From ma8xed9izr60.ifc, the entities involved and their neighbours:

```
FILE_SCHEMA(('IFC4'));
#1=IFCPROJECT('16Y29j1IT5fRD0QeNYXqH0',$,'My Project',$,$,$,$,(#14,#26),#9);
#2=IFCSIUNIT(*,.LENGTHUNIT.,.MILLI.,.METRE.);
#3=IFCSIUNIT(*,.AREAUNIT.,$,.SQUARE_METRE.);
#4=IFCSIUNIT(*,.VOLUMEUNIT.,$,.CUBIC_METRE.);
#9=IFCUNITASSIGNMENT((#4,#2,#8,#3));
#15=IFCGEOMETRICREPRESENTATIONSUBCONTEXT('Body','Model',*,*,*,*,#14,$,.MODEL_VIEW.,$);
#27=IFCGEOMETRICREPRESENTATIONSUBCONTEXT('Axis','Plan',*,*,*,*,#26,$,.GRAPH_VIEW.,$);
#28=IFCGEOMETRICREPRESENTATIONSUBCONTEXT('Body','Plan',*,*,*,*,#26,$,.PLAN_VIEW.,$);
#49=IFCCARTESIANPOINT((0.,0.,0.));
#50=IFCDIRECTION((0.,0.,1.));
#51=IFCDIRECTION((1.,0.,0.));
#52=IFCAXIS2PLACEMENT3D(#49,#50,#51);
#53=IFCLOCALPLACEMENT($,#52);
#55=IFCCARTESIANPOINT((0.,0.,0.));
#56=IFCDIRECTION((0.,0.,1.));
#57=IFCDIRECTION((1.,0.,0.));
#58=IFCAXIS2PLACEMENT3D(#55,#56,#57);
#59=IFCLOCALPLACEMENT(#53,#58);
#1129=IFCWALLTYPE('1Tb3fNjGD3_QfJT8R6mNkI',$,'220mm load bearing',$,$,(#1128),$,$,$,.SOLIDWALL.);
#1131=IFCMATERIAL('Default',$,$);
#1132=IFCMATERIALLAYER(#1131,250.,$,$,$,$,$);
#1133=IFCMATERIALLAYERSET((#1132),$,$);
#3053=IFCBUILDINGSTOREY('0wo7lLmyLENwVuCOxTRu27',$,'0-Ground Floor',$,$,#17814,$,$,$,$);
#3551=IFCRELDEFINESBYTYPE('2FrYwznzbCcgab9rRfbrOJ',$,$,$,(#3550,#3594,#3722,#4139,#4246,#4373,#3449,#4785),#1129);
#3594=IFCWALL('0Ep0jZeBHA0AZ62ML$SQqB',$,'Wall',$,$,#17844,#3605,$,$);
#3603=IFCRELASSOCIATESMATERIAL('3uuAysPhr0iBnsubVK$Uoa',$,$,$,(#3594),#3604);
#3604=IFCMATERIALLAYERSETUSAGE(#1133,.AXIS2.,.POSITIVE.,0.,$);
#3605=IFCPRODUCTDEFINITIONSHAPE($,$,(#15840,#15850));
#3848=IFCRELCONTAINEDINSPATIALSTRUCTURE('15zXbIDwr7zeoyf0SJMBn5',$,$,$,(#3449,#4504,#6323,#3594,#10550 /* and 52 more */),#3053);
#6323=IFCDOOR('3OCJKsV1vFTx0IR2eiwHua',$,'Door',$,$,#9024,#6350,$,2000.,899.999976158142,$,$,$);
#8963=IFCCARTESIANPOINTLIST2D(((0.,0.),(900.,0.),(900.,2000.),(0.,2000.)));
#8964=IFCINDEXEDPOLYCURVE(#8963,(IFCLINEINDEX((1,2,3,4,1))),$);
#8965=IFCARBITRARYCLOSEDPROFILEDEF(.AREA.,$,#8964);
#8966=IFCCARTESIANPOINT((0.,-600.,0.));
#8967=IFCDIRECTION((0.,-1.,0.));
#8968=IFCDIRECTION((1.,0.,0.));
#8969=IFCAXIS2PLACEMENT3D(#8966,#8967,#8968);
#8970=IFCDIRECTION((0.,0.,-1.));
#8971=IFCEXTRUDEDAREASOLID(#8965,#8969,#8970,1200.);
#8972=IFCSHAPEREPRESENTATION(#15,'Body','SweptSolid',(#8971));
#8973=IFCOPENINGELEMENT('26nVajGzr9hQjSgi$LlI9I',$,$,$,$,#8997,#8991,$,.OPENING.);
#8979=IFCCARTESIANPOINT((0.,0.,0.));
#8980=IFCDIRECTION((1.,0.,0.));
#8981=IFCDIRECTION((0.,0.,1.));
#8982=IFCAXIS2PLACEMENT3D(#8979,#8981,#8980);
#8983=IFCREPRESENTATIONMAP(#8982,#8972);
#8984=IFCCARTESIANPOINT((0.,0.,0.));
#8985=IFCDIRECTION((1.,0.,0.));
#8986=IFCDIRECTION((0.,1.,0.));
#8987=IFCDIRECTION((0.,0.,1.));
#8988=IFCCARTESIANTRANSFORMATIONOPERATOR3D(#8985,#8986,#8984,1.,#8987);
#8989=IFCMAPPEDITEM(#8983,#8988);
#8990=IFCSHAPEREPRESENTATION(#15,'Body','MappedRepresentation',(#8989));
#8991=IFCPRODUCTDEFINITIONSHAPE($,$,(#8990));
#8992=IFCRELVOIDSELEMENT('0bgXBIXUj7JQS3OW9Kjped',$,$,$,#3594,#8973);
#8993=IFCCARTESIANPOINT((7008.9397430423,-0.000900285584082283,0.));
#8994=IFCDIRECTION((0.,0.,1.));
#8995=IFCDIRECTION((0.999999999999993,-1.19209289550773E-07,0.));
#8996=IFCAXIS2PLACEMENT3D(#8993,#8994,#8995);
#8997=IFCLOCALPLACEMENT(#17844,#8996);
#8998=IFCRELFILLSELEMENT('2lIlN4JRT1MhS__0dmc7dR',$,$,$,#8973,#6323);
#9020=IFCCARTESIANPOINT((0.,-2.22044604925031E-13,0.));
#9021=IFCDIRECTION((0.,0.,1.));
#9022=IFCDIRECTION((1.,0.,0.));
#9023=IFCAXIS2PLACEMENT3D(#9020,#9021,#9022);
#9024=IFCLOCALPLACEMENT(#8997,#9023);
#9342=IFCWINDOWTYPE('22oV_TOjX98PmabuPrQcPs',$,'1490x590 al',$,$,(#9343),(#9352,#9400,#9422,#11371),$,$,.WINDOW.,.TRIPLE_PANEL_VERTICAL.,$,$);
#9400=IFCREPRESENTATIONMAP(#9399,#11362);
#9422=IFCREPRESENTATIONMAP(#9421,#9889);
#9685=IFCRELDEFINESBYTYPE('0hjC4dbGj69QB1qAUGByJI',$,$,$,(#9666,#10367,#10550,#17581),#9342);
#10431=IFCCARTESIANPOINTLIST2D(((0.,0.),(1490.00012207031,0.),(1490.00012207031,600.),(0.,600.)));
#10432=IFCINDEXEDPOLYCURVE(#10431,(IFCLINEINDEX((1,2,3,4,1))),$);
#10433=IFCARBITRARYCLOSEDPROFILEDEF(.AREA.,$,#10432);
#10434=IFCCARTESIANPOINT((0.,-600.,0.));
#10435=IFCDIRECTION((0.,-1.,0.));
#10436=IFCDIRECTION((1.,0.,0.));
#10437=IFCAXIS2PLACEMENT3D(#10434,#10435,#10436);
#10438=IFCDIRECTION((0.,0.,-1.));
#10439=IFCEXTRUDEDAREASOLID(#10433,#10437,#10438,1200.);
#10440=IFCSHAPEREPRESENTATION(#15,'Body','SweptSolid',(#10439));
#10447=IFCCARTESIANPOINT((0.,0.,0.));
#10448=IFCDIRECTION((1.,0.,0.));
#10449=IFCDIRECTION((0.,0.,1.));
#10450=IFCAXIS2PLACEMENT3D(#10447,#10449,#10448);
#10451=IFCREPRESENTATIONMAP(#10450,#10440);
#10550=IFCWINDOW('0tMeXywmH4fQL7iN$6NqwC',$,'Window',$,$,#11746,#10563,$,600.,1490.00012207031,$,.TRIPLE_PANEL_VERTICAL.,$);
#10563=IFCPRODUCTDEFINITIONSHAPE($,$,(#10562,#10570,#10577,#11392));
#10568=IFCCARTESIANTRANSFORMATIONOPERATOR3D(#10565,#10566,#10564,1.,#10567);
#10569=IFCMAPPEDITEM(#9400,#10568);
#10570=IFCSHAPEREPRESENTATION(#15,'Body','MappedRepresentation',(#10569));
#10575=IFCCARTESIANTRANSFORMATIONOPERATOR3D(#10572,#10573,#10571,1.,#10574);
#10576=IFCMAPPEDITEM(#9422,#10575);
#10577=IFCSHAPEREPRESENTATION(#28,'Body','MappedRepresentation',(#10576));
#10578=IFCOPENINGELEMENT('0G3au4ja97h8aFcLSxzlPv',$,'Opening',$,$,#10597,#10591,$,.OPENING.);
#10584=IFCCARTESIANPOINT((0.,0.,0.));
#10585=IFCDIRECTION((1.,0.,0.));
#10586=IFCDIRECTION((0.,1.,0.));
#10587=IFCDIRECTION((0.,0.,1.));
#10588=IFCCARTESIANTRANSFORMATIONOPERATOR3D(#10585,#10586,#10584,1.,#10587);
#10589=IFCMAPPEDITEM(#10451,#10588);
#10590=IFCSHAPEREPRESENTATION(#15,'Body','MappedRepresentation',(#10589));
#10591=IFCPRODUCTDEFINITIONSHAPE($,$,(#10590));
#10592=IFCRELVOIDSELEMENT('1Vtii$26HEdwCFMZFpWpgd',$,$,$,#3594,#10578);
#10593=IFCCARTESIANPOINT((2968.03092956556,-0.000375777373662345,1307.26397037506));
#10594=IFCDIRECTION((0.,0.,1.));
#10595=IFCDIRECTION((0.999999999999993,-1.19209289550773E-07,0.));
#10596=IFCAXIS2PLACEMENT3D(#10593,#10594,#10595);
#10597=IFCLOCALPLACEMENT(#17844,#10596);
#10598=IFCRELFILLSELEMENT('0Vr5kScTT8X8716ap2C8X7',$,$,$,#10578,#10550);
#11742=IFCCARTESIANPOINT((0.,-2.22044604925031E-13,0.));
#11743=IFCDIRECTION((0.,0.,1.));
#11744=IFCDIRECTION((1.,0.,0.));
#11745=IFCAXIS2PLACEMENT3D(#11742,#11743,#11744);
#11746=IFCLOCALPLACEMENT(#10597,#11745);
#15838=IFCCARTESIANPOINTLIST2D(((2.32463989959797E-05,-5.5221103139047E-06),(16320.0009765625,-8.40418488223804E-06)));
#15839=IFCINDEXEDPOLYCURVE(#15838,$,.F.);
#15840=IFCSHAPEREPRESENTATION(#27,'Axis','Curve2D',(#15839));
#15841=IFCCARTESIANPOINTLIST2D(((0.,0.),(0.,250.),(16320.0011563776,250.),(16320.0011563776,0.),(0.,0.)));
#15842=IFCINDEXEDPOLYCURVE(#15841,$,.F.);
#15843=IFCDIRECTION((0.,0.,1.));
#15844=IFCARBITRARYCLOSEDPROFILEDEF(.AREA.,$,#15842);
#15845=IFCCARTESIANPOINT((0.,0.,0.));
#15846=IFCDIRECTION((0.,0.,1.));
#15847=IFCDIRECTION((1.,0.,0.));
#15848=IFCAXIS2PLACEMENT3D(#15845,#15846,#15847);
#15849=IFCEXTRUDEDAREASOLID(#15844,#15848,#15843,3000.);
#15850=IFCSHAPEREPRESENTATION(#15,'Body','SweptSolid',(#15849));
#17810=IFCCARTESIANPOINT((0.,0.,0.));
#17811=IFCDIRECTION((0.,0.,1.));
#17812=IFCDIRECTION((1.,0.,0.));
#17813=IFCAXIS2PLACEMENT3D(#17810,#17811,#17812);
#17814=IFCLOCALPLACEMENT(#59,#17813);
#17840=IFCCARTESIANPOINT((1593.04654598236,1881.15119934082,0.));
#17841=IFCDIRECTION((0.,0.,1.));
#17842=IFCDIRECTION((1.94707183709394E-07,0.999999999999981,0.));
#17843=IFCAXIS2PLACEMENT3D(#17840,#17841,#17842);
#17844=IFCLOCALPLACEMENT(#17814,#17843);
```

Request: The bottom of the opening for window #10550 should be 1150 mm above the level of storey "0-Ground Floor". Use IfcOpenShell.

```python
import numpy as np
import ifcopenshell
import ifcopenshell.api.geometry
import ifcopenshell.geom
import ifcopenshell.util.element
import ifcopenshell.util.placement
import ifcopenshell.util.shape
import ifcopenshell.util.unit

model = ifcopenshell.open("ma8xed9izr60.ifc")
unit_scale = ifcopenshell.util.unit.calculate_unit_scale(model)

window = model.by_guid("0tMeXywmH4fQL7iN$6NqwC")
opening = window.FillsVoids[0].RelatingOpeningElement
storey = ifcopenshell.util.element.get_container(window, ifc_class="IfcBuildingStorey")
level = ifcopenshell.util.placement.get_local_placement(storey.ObjectPlacement)[2, 3]

# The opening's origin need not be at the sill, so measure its lowest point.
shape = ifcopenshell.geom.create_shape(ifcopenshell.geom.settings(), opening)
bottom = ifcopenshell.util.shape.get_shape_bottom_elevation(shape, shape.geometry) / unit_scale
dz = level + 1150.0 - bottom

shift = np.array([0.0, 0.0, dz])
# The window is placed relative to its opening, so it follows when the opening moves.
matrix = ifcopenshell.util.placement.get_local_placement(opening.ObjectPlacement)
matrix[:3, 3] += shift
ifcopenshell.api.geometry.edit_object_placement(
    model, product=opening, matrix=matrix, is_si=False, should_transform_children=True
)

print(f"moved by {dz * unit_scale:+.3f} m")

model.write("ma8xed9izr60_v2.ifc")
```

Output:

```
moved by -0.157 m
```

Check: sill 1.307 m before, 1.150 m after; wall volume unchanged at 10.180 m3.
